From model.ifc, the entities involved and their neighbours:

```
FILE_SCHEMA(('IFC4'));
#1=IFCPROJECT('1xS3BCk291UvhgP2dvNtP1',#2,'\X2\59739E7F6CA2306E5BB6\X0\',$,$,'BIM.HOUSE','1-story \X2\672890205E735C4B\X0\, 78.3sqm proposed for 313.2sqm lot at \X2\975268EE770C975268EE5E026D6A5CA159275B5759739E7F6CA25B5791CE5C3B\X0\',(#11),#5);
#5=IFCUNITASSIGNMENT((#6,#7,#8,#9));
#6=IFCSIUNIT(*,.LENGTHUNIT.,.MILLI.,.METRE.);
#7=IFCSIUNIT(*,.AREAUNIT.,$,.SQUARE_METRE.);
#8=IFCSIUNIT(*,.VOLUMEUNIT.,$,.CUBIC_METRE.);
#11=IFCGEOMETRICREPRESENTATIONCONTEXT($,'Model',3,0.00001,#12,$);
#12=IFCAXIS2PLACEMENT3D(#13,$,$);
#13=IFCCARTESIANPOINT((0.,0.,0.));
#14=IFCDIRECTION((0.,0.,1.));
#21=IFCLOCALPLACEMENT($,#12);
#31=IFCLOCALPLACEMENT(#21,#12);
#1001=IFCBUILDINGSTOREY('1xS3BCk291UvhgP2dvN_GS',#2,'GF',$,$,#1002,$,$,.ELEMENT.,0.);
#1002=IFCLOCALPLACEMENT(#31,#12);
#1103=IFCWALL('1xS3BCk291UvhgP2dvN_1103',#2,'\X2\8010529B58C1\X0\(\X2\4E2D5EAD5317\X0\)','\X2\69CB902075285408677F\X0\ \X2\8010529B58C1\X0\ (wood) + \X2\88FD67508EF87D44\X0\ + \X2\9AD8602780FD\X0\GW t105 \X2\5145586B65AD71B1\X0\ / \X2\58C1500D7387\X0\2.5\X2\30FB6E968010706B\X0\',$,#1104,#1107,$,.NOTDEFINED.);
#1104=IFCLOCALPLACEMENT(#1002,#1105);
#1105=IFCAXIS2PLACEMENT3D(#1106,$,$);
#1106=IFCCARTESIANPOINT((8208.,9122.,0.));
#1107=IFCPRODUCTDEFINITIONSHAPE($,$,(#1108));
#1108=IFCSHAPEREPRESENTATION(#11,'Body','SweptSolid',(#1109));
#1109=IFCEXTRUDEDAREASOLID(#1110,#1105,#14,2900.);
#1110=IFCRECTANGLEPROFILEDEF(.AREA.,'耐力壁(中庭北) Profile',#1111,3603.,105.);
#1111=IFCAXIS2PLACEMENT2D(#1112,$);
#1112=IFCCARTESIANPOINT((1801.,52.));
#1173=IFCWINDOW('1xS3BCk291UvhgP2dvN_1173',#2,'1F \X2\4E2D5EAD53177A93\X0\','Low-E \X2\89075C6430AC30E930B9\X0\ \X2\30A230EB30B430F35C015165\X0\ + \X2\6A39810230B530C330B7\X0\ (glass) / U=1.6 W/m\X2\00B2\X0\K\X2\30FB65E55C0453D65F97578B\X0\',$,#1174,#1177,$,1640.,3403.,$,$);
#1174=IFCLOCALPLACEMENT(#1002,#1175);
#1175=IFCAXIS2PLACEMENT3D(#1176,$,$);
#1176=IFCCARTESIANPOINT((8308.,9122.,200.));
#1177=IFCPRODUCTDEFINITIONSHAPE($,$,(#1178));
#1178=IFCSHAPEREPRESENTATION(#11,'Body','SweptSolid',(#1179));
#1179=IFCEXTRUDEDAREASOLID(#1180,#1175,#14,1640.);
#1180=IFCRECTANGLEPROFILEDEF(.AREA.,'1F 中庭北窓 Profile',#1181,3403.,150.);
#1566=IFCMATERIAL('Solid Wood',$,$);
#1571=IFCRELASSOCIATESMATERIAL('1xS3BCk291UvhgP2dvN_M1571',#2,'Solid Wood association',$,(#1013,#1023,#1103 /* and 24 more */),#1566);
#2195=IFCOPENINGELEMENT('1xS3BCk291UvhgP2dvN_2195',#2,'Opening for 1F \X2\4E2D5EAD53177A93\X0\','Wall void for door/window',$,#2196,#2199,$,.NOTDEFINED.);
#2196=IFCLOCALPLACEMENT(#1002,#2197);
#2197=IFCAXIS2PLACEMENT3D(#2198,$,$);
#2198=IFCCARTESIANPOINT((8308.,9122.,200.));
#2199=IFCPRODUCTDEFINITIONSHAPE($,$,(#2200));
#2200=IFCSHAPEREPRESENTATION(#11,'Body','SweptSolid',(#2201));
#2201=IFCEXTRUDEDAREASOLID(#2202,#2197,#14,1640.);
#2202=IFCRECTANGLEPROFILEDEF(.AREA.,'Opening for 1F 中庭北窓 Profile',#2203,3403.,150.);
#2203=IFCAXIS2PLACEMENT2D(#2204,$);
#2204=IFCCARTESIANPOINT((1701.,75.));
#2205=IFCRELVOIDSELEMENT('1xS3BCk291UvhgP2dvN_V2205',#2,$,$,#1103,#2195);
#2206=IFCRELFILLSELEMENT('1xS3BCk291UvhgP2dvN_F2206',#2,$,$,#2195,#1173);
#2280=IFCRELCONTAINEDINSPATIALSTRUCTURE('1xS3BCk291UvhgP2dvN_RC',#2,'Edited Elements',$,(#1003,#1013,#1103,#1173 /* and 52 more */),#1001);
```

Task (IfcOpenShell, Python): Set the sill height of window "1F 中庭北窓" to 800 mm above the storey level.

```python
import numpy as np
import ifcopenshell
import ifcopenshell.api.geometry
import ifcopenshell.geom
import ifcopenshell.util.element
import ifcopenshell.util.placement
import ifcopenshell.util.shape
import ifcopenshell.util.unit

model = ifcopenshell.open("model.ifc")
unit_scale = ifcopenshell.util.unit.calculate_unit_scale(model)

window = model.by_guid("1xS3BCk291UvhgP2dvN_1173")
opening = window.FillsVoids[0].RelatingOpeningElement
storey = ifcopenshell.util.element.get_container(window, ifc_class="IfcBuildingStorey")
level = ifcopenshell.util.placement.get_local_placement(storey.ObjectPlacement)[2, 3]

# The opening's origin need not be at the sill, so measure its lowest point.
shape = ifcopenshell.geom.create_shape(ifcopenshell.geom.settings(), opening)
bottom = ifcopenshell.util.shape.get_shape_bottom_elevation(shape, shape.geometry) / unit_scale
dz = level + 800.0 - bottom

shift = np.array([0.0, 0.0, dz])
# The window is not placed relative to its opening, so move both.
for product in (opening, window):
    matrix = ifcopenshell.util.placement.get_local_placement(product.ObjectPlacement)
    matrix[:3, 3] += shift
    ifcopenshell.api.geometry.edit_object_placement(model, product=product, matrix=matrix, is_si=False)

print(f"moved by {dz * unit_scale:+.3f} m")

model.write("model_updated.ifc")
```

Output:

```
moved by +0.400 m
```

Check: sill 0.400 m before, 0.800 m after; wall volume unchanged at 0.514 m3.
